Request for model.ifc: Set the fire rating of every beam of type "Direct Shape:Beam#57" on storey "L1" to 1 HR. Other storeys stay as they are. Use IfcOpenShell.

First a look at what the model holds.

```python
import ifcopenshell
import ifcopenshell.util.element

model = ifcopenshell.open("model.ifc")
print(model.schema)
storey = next(s for s in model.by_type("IfcBuildingStorey") if s.Name == "L1")
beams = [e for e in ifcopenshell.util.element.get_decomposition(storey) if e.is_a("IfcBeam")]
seen = {}
for e in beams:
    element_type = ifcopenshell.util.element.get_type(e)
    key = (element_type.Name if element_type != e and element_type else None, ifcopenshell.util.element.get_pset(e, "Pset_BeamCommon", "FireRating"))
    seen[key] = seen.get(key, 0) + 1
for (name, value), count in sorted(seen.items(), key=str):
    print(count, "x", name, "|", value)
```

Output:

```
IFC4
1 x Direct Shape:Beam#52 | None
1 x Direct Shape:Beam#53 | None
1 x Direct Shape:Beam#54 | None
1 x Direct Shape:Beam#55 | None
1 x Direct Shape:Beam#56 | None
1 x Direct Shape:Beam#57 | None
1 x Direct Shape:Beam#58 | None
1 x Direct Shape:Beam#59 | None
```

```python
import ifcopenshell
import ifcopenshell.api.pset
import ifcopenshell.util.element

model = ifcopenshell.open("model.ifc")

storey = next(s for s in model.by_type("IfcBuildingStorey") if s.Name == "L1")
beams = [e for e in ifcopenshell.util.element.get_decomposition(storey) if e.is_a("IfcBeam")]

count = 0
for e in beams:
    element_type = ifcopenshell.util.element.get_type(e)
    if element_type in (None, e) or element_type.Name != "Direct Shape:Beam#57":
        continue
    # add_pset returns the element's existing set when there is one.
    pset = ifcopenshell.api.pset.add_pset(model, product=e, name="Pset_BeamCommon")
    ifcopenshell.api.pset.edit_pset(model, pset=pset, properties={"FireRating": "1 HR"})
    count += 1

print(count, "beams updated")

model.write("model_v2.ifc")
```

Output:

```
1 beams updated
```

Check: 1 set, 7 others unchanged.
